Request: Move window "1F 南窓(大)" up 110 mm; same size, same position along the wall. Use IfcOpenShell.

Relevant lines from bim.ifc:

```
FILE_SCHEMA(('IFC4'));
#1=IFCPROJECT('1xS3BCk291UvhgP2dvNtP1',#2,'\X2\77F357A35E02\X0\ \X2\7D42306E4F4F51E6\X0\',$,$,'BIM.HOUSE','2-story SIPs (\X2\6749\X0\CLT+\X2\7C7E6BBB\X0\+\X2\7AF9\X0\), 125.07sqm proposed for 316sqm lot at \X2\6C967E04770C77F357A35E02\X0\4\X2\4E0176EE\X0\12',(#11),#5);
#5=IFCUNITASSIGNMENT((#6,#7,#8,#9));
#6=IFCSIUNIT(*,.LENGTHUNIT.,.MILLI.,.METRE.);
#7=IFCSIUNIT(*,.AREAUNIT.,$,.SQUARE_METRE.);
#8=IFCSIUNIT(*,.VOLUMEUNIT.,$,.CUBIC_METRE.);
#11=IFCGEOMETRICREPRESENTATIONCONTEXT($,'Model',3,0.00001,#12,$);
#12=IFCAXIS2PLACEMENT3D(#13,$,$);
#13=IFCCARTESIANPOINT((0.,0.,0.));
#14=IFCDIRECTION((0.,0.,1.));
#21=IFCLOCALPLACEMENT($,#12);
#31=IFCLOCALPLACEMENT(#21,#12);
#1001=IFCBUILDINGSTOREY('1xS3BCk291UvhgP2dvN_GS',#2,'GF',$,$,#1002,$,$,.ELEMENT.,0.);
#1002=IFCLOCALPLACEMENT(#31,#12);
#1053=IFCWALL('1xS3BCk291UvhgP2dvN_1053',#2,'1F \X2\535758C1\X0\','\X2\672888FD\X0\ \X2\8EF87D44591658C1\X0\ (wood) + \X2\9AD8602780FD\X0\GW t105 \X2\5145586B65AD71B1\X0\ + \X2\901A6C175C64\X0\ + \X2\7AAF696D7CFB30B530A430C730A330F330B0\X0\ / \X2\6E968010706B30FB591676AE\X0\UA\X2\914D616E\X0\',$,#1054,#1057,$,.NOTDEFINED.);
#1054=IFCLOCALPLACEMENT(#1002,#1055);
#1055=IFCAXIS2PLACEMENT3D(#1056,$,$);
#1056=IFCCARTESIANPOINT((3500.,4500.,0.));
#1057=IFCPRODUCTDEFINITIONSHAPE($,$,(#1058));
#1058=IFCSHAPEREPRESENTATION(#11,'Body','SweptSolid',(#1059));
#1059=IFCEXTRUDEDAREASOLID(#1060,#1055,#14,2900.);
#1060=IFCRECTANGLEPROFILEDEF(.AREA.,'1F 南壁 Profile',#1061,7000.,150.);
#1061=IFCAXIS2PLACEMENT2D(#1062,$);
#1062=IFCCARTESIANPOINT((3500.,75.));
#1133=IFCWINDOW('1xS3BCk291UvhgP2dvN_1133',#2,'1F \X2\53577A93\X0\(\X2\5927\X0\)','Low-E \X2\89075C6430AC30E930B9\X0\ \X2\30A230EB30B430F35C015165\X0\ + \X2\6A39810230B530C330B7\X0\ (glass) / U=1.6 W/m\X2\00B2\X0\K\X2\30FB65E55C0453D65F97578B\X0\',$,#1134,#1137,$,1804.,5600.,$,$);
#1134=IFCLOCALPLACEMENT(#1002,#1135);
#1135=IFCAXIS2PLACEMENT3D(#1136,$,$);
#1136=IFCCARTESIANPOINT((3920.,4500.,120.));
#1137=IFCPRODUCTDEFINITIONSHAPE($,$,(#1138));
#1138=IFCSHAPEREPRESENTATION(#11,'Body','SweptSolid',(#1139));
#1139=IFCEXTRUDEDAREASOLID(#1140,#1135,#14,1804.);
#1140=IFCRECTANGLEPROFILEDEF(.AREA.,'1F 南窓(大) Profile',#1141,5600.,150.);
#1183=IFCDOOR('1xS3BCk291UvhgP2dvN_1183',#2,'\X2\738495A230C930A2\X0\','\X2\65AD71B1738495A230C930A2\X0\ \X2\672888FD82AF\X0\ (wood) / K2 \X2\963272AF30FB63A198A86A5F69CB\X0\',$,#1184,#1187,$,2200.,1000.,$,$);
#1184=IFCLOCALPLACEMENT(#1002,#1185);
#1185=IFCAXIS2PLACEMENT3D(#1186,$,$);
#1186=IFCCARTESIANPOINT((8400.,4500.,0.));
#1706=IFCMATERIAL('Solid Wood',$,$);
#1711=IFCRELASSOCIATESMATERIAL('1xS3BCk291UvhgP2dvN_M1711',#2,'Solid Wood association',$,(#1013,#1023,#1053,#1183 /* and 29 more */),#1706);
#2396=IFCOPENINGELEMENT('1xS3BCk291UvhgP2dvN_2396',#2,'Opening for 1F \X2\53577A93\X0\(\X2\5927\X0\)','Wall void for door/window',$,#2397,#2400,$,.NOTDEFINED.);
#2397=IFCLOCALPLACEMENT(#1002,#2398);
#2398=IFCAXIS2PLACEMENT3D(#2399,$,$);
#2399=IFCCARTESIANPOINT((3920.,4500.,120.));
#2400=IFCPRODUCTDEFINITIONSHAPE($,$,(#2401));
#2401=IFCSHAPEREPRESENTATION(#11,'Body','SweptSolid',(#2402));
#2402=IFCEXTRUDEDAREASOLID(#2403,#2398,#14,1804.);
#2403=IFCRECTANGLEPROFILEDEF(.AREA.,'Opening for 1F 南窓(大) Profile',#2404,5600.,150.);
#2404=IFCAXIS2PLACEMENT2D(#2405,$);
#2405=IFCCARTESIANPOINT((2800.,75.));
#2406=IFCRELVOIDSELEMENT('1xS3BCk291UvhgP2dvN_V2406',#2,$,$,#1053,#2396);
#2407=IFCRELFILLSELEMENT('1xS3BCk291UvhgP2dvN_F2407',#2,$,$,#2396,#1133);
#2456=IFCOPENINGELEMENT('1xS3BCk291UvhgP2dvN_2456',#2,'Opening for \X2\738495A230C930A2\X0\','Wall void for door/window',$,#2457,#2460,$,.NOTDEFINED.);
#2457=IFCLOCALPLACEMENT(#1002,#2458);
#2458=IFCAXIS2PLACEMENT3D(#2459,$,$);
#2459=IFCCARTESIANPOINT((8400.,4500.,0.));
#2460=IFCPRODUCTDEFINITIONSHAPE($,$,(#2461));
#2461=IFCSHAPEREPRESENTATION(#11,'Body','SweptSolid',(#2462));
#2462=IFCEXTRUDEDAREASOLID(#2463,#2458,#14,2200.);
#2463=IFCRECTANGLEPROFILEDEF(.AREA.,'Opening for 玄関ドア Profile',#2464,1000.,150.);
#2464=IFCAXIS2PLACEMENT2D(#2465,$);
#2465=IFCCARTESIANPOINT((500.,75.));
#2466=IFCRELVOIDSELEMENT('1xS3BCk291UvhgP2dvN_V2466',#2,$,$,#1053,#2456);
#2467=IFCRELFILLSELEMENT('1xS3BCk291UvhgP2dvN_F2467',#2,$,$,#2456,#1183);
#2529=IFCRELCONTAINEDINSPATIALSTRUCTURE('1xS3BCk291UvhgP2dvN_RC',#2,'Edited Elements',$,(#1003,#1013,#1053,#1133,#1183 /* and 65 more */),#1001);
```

```python
import numpy as np
import ifcopenshell
import ifcopenshell.api.geometry
import ifcopenshell.util.placement
import ifcopenshell.util.unit

model = ifcopenshell.open("bim.ifc")
unit_scale = ifcopenshell.util.unit.calculate_unit_scale(model)

window = model.by_id(1133)
opening = window.FillsVoids[0].RelatingOpeningElement
dz = 0.11 / unit_scale

shift = np.array([0.0, 0.0, dz])
# The window is not placed relative to its opening, so move both.
for product in (opening, window):
    matrix = ifcopenshell.util.placement.get_local_placement(product.ObjectPlacement)
    matrix[:3, 3] += shift
    ifcopenshell.api.geometry.edit_object_placement(model, product=product, matrix=matrix, is_si=False)

print(f"moved by {dz * unit_scale:+.3f} m")

model.write("bim-out.ifc")
```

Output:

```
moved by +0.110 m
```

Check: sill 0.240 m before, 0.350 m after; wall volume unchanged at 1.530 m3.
